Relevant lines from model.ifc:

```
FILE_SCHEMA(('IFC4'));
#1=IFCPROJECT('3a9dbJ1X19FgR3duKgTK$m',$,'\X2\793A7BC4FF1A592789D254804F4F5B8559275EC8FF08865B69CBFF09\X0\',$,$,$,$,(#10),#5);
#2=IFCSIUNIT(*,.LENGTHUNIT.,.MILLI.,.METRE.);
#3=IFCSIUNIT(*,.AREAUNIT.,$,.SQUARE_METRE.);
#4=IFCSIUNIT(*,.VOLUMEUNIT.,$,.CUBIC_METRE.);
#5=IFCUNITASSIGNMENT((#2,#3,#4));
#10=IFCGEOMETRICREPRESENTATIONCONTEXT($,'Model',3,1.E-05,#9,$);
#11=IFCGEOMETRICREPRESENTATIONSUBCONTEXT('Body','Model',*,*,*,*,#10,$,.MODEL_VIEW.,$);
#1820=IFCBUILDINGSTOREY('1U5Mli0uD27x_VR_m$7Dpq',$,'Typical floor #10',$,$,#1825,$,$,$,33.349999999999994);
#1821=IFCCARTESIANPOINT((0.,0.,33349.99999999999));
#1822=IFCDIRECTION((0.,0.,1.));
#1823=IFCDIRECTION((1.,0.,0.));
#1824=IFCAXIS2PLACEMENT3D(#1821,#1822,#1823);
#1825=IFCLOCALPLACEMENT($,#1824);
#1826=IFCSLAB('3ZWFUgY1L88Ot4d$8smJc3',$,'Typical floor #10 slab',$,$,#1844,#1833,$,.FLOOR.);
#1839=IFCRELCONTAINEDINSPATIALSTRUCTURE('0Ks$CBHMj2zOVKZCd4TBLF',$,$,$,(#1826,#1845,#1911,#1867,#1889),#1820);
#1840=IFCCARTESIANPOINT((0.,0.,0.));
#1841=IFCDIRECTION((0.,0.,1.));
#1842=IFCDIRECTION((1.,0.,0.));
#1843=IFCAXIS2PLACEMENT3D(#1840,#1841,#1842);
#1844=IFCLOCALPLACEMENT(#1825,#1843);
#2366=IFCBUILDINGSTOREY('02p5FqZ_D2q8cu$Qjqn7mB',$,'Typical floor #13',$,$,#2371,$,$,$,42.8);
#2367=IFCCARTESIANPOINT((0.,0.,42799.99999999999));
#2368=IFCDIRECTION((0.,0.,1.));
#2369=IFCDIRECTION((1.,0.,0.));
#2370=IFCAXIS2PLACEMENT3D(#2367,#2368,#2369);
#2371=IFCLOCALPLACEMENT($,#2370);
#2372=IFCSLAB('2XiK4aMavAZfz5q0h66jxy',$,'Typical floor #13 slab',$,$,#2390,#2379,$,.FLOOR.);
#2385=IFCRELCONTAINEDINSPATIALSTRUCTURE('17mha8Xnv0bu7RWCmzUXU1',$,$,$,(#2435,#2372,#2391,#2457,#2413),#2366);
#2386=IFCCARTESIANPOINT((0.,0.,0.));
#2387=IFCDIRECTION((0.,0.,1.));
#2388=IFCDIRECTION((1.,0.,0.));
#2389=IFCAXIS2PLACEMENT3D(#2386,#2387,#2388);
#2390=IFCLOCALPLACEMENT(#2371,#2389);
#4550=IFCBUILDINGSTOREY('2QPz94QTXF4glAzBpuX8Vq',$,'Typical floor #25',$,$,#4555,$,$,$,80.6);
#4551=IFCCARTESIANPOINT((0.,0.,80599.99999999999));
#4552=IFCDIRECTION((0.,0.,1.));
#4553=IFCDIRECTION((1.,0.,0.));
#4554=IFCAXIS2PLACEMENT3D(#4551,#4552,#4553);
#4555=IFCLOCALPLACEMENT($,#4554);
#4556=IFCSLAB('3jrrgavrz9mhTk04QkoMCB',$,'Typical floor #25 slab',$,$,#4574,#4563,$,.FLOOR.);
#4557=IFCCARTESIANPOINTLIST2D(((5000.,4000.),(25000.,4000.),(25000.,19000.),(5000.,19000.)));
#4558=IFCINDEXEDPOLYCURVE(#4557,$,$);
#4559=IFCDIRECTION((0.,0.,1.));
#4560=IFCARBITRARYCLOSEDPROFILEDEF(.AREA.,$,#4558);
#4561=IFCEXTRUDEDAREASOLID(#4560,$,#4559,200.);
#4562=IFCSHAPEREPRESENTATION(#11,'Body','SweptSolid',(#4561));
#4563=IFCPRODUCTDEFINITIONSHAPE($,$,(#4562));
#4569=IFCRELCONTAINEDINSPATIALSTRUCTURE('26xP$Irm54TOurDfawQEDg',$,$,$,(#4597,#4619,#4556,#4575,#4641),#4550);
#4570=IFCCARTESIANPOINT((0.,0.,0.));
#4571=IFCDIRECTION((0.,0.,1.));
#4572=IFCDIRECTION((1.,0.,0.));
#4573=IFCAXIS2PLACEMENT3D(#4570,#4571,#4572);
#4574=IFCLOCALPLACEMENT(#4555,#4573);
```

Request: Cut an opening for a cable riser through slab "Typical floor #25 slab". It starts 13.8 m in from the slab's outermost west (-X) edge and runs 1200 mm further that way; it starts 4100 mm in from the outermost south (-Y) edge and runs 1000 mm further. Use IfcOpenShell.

```python
import numpy as np
import ifcopenshell
import ifcopenshell.api.feature
import ifcopenshell.api.geometry
import ifcopenshell.api.root
import ifcopenshell.geom
import ifcopenshell.util.placement
import ifcopenshell.util.representation
import ifcopenshell.util.shape
import ifcopenshell.util.unit

model = ifcopenshell.open("model.ifc")
unit_scale = ifcopenshell.util.unit.calculate_unit_scale(model)
settings = ifcopenshell.geom.settings()


def volume(element):
    """Net volume in cubic metres, openings subtracted."""
    shape = ifcopenshell.geom.create_shape(settings, element)
    return ifcopenshell.util.shape.get_volume(shape.geometry)


slab = model.by_guid("3jrrgavrz9mhTk04QkoMCB")
before = volume(slab)

# Extent in the slab's own axes, in metres. The edges named are its -X and -Y sides.
slab_shape = ifcopenshell.geom.create_shape(settings, slab)
vertices = ifcopenshell.util.shape.get_vertices(slab_shape.geometry)
x_min, y_min, bottom = vertices.min(axis=0)
top = vertices[:, 2].max()

opening = ifcopenshell.api.root.create_entity(model, ifc_class="IfcOpeningElement", name="Cable riser opening", predefined_type="OPENING")
context = ifcopenshell.util.representation.get_context(model, "Model", "Body", "MODEL_VIEW")
width, depth = 1.2, 1
outline = [(0.0, 0.0), (width, 0.0), (width, depth), (0.0, depth), (0.0, 0.0)]
# Overshoot both faces by 50 mm so the cut is clean.
shape = ifcopenshell.api.geometry.add_slab_representation(
    model, context=context, depth=top - bottom + 0.1, polyline=outline
)
ifcopenshell.api.geometry.assign_representation(model, product=opening, representation=shape)

matrix = ifcopenshell.util.placement.get_local_placement(slab.ObjectPlacement)
matrix[:, 3] = matrix @ np.append(np.array([x_min + 13.8, y_min + 4.1, bottom - 0.05]) / unit_scale, 1.0)
ifcopenshell.api.geometry.edit_object_placement(model, product=opening, matrix=matrix, is_si=False)
ifcopenshell.api.feature.add_feature(model, feature=opening, element=slab)

after = volume(slab)

print(f"slab volume {before:.3f} -> {after:.3f} m3")

model.write("model_v2.ifc")
```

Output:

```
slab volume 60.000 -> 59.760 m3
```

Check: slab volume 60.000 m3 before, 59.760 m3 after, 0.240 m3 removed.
